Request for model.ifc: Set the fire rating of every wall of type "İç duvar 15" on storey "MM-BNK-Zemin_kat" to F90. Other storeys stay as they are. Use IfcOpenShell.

First a look at what the model holds.

```python
import ifcopenshell
import ifcopenshell.util.element

model = ifcopenshell.open("model.ifc")
print(model.schema)
storey = next(s for s in model.by_type("IfcBuildingStorey") if s.Name == "MM-BNK-Zemin_kat")
walls = [e for e in ifcopenshell.util.element.get_decomposition(storey) if e.is_a("IfcWall")]
seen = {}
for e in walls:
    element_type = ifcopenshell.util.element.get_type(e)
    key = (element_type.Name if element_type != e and element_type else None, ifcopenshell.util.element.get_pset(e, "Pset_WallCommon", "FireRating"))
    seen[key] = seen.get(key, 0) + 1
for (name, value), count in sorted(seen.items(), key=str):
    print(count, "x", name, "|", value)
```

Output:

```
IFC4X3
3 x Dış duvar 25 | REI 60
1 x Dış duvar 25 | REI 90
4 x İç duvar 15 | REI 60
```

```python
import ifcopenshell
import ifcopenshell.api.pset
import ifcopenshell.util.element

model = ifcopenshell.open("model.ifc")

storey = next(s for s in model.by_type("IfcBuildingStorey") if s.Name == "MM-BNK-Zemin_kat")
walls = [e for e in ifcopenshell.util.element.get_decomposition(storey) if e.is_a("IfcWall")]

count = 0
for e in walls:
    element_type = ifcopenshell.util.element.get_type(e)
    if element_type in (None, e) or element_type.Name != "İç duvar 15":
        continue
    # add_pset returns the element's existing set when there is one.
    pset = ifcopenshell.api.pset.add_pset(model, product=e, name="Pset_WallCommon")
    ifcopenshell.api.pset.edit_pset(model, pset=pset, properties={"FireRating": "F90"})
    count += 1

print(count, "walls updated")

model.write("model_updated.ifc")
```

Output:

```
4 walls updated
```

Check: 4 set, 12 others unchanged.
